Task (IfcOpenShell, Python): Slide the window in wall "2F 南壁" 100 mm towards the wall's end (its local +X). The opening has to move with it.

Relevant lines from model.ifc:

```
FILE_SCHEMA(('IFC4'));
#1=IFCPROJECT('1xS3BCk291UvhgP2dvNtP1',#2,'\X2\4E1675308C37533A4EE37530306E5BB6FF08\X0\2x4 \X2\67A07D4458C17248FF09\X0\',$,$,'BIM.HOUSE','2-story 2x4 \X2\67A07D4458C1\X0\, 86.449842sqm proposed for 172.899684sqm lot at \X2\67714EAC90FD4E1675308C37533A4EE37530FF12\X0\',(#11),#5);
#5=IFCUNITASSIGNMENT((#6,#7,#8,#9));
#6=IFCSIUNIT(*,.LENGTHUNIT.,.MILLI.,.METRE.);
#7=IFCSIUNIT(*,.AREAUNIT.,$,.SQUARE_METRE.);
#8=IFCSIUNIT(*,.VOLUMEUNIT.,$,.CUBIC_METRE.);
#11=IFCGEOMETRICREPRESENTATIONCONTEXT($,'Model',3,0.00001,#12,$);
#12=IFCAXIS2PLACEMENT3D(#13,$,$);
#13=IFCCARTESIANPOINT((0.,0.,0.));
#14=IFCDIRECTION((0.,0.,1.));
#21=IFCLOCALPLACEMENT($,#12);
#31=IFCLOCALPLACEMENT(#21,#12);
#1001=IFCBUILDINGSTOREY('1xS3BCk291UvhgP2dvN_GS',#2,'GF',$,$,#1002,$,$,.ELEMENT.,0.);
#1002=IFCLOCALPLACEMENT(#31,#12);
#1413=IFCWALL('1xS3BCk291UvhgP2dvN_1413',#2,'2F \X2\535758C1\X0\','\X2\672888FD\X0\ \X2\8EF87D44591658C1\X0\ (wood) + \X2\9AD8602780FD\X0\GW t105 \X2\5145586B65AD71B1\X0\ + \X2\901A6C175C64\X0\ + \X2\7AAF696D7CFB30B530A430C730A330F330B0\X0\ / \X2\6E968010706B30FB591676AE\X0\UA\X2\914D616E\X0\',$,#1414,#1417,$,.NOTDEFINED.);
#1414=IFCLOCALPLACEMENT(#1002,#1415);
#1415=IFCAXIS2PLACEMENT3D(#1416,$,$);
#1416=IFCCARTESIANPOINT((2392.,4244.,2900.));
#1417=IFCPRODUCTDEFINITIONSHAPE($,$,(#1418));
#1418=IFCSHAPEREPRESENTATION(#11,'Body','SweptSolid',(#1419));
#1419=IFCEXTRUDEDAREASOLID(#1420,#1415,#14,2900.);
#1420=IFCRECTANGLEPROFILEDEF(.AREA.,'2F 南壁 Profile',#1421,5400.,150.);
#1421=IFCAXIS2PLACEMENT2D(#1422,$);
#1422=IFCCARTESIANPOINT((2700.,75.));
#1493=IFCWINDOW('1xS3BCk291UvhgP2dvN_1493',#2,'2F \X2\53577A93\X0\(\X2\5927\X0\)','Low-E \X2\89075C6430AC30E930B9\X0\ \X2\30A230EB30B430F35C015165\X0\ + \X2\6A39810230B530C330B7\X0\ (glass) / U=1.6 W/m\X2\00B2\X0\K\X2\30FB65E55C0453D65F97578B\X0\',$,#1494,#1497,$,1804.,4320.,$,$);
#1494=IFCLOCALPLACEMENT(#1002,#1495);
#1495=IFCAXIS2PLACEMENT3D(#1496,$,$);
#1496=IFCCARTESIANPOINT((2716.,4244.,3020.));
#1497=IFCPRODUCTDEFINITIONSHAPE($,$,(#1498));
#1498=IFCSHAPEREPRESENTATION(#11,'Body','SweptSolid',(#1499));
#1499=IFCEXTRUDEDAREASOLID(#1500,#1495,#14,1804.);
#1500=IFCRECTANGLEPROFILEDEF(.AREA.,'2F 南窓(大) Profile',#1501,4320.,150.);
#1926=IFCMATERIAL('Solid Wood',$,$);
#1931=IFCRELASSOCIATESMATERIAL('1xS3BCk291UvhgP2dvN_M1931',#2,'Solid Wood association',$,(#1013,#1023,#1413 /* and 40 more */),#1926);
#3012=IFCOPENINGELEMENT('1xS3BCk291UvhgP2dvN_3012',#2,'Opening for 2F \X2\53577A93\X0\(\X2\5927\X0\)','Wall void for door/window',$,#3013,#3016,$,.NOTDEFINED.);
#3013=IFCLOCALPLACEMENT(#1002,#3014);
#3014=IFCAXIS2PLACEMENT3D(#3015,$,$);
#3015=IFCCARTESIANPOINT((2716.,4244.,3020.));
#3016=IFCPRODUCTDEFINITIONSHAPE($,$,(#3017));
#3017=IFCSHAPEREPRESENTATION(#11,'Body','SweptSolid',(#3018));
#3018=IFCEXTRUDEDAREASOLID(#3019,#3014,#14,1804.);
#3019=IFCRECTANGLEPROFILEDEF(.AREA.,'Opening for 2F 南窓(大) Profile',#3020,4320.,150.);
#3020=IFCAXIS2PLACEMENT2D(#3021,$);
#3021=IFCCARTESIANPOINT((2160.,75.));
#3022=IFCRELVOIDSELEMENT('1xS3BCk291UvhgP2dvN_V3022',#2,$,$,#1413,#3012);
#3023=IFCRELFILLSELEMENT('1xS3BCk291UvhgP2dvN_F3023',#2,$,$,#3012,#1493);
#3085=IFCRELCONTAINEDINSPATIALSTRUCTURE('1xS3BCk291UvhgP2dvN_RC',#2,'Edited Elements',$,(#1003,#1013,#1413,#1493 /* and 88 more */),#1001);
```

```python
import ifcopenshell
import ifcopenshell.api.geometry
import ifcopenshell.util.placement

model = ifcopenshell.open("model.ifc")

window = model.by_guid("1xS3BCk291UvhgP2dvN_1493")
opening = window.FillsVoids[0].RelatingOpeningElement
wall = opening.VoidsElements[0].RelatingBuildingElement

wall_matrix = ifcopenshell.util.placement.get_local_placement(wall.ObjectPlacement)
shift = wall_matrix[:3, 0] * 100.0
before = ifcopenshell.util.placement.get_local_placement(window.ObjectPlacement)[:3, 3].copy()

# The window is not placed relative to its opening, so move both.
for product in (opening, window):
    matrix = ifcopenshell.util.placement.get_local_placement(product.ObjectPlacement)
    matrix[:3, 3] += shift
    ifcopenshell.api.geometry.edit_object_placement(model, product=product, matrix=matrix, is_si=False)

after = ifcopenshell.util.placement.get_local_placement(window.ObjectPlacement)[:3, 3]
print("window moved by", (after - before).round(3) + 0.0)

model.write("model_v2.ifc")
```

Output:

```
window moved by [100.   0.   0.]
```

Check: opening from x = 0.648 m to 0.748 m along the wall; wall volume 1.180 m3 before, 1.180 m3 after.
